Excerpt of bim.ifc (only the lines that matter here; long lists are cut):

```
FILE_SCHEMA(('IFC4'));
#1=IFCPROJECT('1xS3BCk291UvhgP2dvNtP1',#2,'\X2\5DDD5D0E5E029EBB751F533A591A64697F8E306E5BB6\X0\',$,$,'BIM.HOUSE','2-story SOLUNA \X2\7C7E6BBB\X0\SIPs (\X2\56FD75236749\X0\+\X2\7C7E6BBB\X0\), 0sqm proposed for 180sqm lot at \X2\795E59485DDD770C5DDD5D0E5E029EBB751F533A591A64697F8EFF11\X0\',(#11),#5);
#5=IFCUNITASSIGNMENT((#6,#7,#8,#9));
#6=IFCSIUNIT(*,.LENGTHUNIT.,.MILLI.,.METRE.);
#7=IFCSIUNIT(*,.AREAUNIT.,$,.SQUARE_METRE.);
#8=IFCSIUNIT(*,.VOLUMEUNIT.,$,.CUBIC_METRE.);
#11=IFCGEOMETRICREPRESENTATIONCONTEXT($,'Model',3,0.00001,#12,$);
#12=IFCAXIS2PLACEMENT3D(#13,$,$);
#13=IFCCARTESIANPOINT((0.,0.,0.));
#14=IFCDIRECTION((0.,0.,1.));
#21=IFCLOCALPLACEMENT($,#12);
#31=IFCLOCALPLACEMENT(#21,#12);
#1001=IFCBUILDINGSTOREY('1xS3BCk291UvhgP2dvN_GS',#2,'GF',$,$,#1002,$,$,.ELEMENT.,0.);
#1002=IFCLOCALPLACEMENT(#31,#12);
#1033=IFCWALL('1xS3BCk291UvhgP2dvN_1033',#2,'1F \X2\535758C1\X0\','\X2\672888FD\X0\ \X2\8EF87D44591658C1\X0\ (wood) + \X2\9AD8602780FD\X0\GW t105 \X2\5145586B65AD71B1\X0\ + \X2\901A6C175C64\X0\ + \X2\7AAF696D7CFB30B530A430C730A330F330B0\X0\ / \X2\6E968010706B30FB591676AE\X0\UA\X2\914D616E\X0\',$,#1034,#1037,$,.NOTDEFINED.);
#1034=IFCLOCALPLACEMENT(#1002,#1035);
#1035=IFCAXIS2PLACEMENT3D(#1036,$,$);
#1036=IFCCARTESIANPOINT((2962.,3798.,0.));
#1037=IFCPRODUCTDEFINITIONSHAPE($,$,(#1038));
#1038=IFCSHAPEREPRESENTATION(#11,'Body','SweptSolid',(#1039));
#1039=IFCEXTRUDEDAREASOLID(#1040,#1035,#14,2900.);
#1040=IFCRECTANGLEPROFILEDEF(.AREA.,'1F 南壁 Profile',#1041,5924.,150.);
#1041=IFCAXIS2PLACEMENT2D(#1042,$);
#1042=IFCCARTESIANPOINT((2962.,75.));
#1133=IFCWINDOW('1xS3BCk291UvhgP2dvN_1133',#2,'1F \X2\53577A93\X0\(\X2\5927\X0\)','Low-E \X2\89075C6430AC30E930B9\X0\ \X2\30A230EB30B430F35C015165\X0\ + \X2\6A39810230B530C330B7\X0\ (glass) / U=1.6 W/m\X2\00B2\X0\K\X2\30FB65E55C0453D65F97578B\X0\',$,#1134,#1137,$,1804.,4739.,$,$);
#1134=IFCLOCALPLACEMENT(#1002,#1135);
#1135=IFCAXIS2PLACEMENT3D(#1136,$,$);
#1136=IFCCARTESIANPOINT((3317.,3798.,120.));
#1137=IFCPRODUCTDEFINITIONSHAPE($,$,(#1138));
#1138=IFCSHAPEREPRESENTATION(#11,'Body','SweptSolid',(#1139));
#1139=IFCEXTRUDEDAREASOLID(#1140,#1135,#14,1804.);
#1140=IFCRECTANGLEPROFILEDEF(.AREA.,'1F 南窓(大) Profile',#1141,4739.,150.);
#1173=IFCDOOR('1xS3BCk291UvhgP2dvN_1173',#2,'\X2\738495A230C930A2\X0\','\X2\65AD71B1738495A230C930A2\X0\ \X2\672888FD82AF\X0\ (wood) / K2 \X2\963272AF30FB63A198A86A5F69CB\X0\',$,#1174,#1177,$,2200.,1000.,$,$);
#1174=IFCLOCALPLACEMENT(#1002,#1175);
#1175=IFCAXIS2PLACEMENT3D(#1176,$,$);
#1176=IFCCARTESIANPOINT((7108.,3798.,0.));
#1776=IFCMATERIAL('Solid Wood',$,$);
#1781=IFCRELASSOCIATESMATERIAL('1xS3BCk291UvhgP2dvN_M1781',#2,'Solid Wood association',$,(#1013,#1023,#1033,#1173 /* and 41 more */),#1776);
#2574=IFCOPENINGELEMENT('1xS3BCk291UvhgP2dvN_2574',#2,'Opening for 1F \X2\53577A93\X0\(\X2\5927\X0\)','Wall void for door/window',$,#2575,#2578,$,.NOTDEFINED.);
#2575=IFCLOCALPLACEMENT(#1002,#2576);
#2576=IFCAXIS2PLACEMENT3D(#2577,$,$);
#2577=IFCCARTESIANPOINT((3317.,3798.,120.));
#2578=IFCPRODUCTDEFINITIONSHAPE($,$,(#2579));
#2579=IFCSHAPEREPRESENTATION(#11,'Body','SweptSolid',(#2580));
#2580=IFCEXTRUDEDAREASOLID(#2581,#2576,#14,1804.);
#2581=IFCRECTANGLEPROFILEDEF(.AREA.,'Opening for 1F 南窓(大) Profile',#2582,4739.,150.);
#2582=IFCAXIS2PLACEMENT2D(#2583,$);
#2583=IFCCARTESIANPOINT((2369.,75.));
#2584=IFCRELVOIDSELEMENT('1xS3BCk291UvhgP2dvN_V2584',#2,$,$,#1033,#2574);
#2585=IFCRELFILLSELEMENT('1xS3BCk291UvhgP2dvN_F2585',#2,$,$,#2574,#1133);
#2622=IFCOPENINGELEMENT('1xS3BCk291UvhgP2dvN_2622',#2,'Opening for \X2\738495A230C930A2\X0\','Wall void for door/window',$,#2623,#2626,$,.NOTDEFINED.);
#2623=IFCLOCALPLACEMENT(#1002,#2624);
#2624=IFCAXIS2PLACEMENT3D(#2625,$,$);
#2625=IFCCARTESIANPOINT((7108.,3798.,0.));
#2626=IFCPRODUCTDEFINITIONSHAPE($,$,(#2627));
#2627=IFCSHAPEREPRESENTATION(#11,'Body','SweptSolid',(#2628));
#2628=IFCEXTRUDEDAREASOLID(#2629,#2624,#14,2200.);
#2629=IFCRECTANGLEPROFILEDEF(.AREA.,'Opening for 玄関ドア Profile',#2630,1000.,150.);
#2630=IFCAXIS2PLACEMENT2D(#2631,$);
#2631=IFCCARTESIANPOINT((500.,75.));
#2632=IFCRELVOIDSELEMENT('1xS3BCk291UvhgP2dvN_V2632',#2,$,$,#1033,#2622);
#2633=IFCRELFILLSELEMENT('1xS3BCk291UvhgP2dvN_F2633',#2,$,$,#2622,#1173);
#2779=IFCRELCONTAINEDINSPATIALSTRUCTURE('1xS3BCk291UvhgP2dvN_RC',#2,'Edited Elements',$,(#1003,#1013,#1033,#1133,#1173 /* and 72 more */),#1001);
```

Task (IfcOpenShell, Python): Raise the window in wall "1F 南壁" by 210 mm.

```python
import numpy as np
import ifcopenshell
import ifcopenshell.api.geometry
import ifcopenshell.util.placement
import ifcopenshell.util.unit

model = ifcopenshell.open("bim.ifc")
unit_scale = ifcopenshell.util.unit.calculate_unit_scale(model)

window = model.by_guid("1xS3BCk291UvhgP2dvN_1133")
opening = window.FillsVoids[0].RelatingOpeningElement
dz = 210.0

shift = np.array([0.0, 0.0, dz])
# The window is not placed relative to its opening, so move both.
for product in (opening, window):
    matrix = ifcopenshell.util.placement.get_local_placement(product.ObjectPlacement)
    matrix[:3, 3] += shift
    ifcopenshell.api.geometry.edit_object_placement(model, product=product, matrix=matrix, is_si=False)

print(f"moved by {dz * unit_scale:+.3f} m")

model.write("bim_rev.ifc")
```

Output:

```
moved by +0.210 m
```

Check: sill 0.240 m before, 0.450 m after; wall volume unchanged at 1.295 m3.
